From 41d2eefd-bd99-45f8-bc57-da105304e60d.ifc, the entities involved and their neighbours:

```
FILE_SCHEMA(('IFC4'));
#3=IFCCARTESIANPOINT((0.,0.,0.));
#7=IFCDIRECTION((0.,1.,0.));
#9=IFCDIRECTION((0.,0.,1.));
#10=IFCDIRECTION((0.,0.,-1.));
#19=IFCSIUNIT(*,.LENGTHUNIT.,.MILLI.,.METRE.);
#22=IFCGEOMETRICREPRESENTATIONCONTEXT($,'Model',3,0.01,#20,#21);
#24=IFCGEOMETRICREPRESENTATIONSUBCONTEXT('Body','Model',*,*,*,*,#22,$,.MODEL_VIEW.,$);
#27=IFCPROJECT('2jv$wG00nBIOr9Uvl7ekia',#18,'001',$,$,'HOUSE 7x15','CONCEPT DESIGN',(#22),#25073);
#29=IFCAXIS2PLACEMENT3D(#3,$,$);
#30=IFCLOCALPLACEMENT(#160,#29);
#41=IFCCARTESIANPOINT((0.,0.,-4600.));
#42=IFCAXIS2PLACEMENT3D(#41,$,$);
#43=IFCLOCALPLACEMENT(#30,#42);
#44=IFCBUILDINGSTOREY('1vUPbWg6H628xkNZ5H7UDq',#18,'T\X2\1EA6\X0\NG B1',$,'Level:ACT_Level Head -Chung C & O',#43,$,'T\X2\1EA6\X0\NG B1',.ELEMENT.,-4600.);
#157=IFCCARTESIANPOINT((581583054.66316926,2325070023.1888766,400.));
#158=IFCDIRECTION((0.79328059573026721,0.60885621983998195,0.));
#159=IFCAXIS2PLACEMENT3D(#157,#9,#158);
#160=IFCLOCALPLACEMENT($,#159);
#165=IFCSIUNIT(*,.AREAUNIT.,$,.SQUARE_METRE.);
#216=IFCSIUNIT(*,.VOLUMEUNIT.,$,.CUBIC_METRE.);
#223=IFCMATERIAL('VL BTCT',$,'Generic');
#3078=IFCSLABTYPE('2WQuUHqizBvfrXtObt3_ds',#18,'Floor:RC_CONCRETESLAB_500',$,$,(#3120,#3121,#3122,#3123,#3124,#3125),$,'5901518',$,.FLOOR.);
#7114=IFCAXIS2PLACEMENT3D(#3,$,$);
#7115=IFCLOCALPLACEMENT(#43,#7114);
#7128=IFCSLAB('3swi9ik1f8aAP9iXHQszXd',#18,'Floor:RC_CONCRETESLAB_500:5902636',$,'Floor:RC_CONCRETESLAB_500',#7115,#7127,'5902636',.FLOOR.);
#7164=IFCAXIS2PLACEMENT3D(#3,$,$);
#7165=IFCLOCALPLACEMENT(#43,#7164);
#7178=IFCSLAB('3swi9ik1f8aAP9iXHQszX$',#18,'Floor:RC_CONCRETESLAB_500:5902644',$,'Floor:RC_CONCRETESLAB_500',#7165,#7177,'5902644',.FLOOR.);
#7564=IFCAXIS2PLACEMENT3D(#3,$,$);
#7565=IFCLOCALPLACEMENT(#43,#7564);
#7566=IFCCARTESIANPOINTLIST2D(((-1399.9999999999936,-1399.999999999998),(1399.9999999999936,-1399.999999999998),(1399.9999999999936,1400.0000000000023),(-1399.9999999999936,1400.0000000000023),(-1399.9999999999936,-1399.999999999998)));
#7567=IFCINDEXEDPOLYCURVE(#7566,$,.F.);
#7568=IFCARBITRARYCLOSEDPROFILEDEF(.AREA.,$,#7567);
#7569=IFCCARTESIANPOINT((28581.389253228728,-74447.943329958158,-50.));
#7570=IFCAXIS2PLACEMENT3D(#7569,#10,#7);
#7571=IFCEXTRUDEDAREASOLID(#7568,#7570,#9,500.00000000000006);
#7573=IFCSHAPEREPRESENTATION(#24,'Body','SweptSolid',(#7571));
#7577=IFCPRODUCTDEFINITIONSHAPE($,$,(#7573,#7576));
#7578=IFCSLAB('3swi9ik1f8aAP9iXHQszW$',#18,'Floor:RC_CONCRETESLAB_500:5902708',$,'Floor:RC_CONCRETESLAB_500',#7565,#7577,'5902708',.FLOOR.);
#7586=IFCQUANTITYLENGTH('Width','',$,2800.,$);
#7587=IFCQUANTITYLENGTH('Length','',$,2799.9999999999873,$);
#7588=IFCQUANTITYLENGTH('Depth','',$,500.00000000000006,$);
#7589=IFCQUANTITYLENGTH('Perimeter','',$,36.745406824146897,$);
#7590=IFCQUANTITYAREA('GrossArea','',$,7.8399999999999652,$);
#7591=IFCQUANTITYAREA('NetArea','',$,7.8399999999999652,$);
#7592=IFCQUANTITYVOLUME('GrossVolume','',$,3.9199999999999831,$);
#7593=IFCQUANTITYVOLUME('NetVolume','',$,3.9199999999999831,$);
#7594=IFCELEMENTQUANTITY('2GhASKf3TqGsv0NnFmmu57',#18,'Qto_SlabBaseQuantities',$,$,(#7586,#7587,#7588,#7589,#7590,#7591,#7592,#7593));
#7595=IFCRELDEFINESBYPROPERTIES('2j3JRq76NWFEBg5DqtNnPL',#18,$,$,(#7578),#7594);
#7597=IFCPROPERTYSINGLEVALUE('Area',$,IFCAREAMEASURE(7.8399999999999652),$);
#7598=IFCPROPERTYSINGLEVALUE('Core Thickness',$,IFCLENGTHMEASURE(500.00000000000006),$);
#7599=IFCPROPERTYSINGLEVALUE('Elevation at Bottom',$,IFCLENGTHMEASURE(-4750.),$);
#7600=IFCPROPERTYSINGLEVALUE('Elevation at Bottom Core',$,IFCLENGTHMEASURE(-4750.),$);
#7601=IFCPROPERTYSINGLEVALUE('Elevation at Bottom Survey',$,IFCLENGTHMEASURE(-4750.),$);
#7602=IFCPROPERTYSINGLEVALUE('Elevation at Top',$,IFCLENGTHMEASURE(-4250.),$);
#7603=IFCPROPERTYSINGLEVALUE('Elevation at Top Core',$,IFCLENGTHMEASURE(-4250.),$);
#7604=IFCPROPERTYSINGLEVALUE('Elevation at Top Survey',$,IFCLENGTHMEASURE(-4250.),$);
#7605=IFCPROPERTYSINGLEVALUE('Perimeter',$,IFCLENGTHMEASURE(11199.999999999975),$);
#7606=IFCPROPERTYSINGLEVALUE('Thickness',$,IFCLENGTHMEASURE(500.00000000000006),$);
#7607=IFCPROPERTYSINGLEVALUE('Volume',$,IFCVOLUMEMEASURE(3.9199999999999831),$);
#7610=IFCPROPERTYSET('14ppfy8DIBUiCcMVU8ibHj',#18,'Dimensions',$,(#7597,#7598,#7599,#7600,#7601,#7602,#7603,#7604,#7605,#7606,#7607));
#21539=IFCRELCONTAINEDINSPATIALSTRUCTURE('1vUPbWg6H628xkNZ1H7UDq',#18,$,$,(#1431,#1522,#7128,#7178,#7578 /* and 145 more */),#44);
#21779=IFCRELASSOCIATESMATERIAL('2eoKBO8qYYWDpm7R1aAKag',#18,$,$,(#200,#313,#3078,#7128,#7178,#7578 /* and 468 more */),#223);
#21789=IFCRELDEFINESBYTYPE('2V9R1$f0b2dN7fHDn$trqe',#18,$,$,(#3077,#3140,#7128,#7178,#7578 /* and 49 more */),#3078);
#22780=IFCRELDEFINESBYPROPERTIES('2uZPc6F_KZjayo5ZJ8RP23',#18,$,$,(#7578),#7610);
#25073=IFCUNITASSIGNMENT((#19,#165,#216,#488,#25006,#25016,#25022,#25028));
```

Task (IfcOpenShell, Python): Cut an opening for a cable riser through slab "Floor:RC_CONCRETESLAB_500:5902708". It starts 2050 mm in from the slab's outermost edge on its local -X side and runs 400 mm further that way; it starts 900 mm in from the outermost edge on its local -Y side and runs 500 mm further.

```python
import numpy as np
import ifcopenshell
import ifcopenshell.api.feature
import ifcopenshell.api.geometry
import ifcopenshell.api.pset
import ifcopenshell.api.root
import ifcopenshell.geom
import ifcopenshell.util.element
import ifcopenshell.util.placement
import ifcopenshell.util.representation
import ifcopenshell.util.shape
import ifcopenshell.util.unit

model = ifcopenshell.open("41d2eefd-bd99-45f8-bc57-da105304e60d.ifc")
unit_scale = ifcopenshell.util.unit.calculate_unit_scale(model)
area_scale = ifcopenshell.util.unit.calculate_unit_scale(model, "AREAUNIT")
volume_scale = ifcopenshell.util.unit.calculate_unit_scale(model, "VOLUMEUNIT")
settings = ifcopenshell.geom.settings()


def volume(element):
    """Net volume in cubic metres, openings subtracted."""
    shape = ifcopenshell.geom.create_shape(settings, element)
    return ifcopenshell.util.shape.get_volume(shape.geometry)


slab = model.by_guid("3swi9ik1f8aAP9iXHQszW$")
before = volume(slab)

# Extent in the slab's own axes, in metres. The edges named are its -X and -Y sides.
slab_shape = ifcopenshell.geom.create_shape(settings, slab)
vertices = ifcopenshell.util.shape.get_vertices(slab_shape.geometry)
x_min, y_min, bottom = vertices.min(axis=0)
top = vertices[:, 2].max()

opening = ifcopenshell.api.root.create_entity(model, ifc_class="IfcOpeningElement", name="Cable riser opening", predefined_type="OPENING")
context = ifcopenshell.util.representation.get_context(model, "Model", "Body", "MODEL_VIEW")
width, depth = 0.4, 0.5
outline = [(0.0, 0.0), (width, 0.0), (width, depth), (0.0, depth), (0.0, 0.0)]
# Overshoot both faces by 50 mm so the cut is clean.
shape = ifcopenshell.api.geometry.add_slab_representation(
    model, context=context, depth=top - bottom + 0.1, polyline=outline
)
ifcopenshell.api.geometry.assign_representation(model, product=opening, representation=shape)

matrix = ifcopenshell.util.placement.get_local_placement(slab.ObjectPlacement)
matrix[:, 3] = matrix @ np.append(np.array([x_min + 2.05, y_min + 0.9, bottom - 0.05]) / unit_scale, 1.0)
ifcopenshell.api.geometry.edit_object_placement(model, product=opening, matrix=matrix, is_si=False)
ifcopenshell.api.feature.add_feature(model, feature=opening, element=slab)

after = volume(slab)

# Update the slab's stored quantities.
qto = model.by_id(ifcopenshell.util.element.get_pset(slab, "Qto_SlabBaseQuantities", should_inherit=False)["id"])
ifcopenshell.api.pset.edit_qto(model, qto=qto, properties={
    "NetArea": after / (top - bottom) / area_scale,
    "NetVolume": after / volume_scale,
})
pset = model.by_id(ifcopenshell.util.element.get_pset(slab, "Dimensions", should_inherit=False)["id"])
ifcopenshell.api.pset.edit_pset(model, pset=pset, properties={
    "Area": model.create_entity("IfcAreaMeasure", after / (top - bottom) / area_scale),
    "Volume": model.create_entity("IfcVolumeMeasure", after / volume_scale),
})

print(f"slab volume {before:.3f} -> {after:.3f} m3")

model.write("41d2eefd-bd99-45f8-bc57-da105304e60d_edited.ifc")
```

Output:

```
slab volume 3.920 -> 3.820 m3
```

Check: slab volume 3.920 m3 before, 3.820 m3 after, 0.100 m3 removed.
